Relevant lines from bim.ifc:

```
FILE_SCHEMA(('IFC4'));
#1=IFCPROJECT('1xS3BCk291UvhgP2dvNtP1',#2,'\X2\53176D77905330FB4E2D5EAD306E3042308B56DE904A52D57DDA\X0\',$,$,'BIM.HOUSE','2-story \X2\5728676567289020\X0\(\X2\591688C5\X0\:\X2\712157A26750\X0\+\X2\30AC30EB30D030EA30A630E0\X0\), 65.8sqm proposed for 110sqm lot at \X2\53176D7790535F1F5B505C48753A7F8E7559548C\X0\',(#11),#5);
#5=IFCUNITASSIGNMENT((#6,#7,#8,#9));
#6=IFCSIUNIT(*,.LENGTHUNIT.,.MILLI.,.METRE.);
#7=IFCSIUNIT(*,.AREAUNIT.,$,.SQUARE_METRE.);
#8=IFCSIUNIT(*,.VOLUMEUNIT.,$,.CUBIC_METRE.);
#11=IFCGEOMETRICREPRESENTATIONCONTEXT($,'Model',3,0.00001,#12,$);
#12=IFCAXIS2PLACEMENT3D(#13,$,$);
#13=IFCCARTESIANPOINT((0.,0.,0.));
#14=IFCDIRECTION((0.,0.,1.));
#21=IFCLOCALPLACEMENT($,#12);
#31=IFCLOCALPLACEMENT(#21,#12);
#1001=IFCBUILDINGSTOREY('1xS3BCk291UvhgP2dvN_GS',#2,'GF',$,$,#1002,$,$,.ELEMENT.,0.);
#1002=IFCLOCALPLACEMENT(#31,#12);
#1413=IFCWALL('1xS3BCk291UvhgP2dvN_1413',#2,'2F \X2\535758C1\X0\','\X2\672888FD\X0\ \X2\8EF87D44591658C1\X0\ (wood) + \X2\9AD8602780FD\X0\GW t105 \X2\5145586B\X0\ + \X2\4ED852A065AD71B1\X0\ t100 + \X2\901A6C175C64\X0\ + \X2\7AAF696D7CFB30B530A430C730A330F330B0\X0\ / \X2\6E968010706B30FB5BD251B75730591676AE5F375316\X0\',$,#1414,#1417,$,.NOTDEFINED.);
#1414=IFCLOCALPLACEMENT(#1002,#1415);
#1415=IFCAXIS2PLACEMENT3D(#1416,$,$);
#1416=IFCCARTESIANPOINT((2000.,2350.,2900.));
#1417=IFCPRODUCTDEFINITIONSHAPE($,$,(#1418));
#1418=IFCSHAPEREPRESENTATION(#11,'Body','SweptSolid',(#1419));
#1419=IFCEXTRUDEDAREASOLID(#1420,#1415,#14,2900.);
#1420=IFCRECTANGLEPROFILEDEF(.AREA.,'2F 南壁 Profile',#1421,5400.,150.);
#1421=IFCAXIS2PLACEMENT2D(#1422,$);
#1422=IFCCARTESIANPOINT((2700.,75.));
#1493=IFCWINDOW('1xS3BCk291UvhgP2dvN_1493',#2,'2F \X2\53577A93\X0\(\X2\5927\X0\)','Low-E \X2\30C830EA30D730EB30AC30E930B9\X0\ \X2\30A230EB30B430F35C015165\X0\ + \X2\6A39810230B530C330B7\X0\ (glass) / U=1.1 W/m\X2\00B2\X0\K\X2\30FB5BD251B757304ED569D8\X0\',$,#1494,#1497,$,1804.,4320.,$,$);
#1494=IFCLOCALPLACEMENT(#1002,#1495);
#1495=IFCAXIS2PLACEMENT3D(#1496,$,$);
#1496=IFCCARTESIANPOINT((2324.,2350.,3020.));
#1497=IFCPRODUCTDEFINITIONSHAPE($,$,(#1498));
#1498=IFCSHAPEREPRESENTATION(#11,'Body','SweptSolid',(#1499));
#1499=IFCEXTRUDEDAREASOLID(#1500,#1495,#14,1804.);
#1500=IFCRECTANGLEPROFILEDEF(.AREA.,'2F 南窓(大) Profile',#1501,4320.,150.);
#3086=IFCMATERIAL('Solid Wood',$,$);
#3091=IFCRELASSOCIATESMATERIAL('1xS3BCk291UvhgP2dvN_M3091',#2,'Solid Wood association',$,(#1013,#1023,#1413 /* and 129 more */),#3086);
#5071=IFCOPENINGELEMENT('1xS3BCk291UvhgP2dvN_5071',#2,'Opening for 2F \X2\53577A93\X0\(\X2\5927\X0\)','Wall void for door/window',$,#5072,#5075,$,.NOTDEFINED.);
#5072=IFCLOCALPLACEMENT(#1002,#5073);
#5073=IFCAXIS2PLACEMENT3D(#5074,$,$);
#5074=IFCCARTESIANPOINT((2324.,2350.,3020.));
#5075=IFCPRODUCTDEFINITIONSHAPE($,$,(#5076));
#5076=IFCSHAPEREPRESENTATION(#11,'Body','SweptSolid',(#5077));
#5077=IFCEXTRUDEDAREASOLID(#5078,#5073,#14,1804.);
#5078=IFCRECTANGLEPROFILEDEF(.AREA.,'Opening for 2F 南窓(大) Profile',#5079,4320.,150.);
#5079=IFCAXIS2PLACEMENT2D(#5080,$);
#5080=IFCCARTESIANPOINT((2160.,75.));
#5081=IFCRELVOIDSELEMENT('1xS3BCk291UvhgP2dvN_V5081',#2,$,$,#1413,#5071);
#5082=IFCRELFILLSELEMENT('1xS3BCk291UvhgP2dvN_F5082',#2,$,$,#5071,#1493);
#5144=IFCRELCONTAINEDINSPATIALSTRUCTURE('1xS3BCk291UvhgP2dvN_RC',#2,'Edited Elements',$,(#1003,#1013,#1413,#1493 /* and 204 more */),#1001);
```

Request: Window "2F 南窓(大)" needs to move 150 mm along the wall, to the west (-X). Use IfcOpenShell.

```python
import ifcopenshell
import ifcopenshell.api.geometry
import ifcopenshell.util.placement

model = ifcopenshell.open("bim.ifc")

window = model.by_guid("1xS3BCk291UvhgP2dvN_1493")
opening = window.FillsVoids[0].RelatingOpeningElement
wall = opening.VoidsElements[0].RelatingBuildingElement

wall_matrix = ifcopenshell.util.placement.get_local_placement(wall.ObjectPlacement)
shift = wall_matrix[:3, 0] * -150.0
before = ifcopenshell.util.placement.get_local_placement(window.ObjectPlacement)[:3, 3].copy()

# The window is not placed relative to its opening, so move both.
for product in (opening, window):
    matrix = ifcopenshell.util.placement.get_local_placement(product.ObjectPlacement)
    matrix[:3, 3] += shift
    ifcopenshell.api.geometry.edit_object_placement(model, product=product, matrix=matrix, is_si=False)

after = ifcopenshell.util.placement.get_local_placement(window.ObjectPlacement)[:3, 3]
print("window moved by", (after - before).round(3) + 0.0)

model.write("bim-out.ifc")
```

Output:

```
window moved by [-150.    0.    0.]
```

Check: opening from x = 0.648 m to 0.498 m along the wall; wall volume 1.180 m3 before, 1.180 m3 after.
